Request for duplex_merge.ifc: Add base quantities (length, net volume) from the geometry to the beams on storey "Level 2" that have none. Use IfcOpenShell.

First a look at what the model holds.

```python
import ifcopenshell
import ifcopenshell.util.element
import ifcopenshell.util.unit

model = ifcopenshell.open("duplex_merge.ifc")
print(model.schema)
for unit_type in ("LENGTHUNIT", "AREAUNIT", "VOLUMEUNIT"):
    print(unit_type, ifcopenshell.util.unit.calculate_unit_scale(model, unit_type))
storey = next(s for s in model.by_type("IfcBuildingStorey") if s.Name == "Level 2")
beams = [e for e in ifcopenshell.util.element.get_decomposition(storey) if e.is_a("IfcBeam")]
for e in sorted(beams, key=lambda e: e.id()):
    print(e.id(), e.is_a(), e.Name, list(ifcopenshell.util.element.get_psets(e, qtos_only=True)), sep=" | ")
```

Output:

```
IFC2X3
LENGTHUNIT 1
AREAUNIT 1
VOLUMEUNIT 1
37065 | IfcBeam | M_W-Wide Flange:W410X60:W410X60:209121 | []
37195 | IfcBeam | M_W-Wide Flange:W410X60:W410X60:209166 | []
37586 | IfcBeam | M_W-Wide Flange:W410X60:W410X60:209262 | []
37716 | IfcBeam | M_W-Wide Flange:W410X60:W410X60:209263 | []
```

```python
import ifcopenshell
import ifcopenshell.api.pset
import ifcopenshell.geom
import ifcopenshell.util.element
import ifcopenshell.util.shape
import ifcopenshell.util.unit

model = ifcopenshell.open("duplex_merge.ifc")
unit_scale = ifcopenshell.util.unit.calculate_unit_scale(model)
volume_scale = ifcopenshell.util.unit.calculate_unit_scale(model, "VOLUMEUNIT")
settings = ifcopenshell.geom.settings()

storey = next(s for s in model.by_type("IfcBuildingStorey") if s.Name == "Level 2")
beams = [e for e in ifcopenshell.util.element.get_decomposition(storey) if e.is_a("IfcBeam")]

for e in sorted(beams, key=lambda e: e.id()):
    if ifcopenshell.util.element.get_psets(e, qtos_only=True, should_inherit=False):
        continue
    # Geometry comes back in metres, in the element's own axes.
    shape = ifcopenshell.geom.create_shape(settings, e)
    values = {
        "Length": ifcopenshell.util.shape.get_max_xyz(shape.geometry) / unit_scale,
        "NetVolume": ifcopenshell.util.shape.get_volume(shape.geometry) / volume_scale,
    }
    qto = ifcopenshell.api.pset.add_qto(model, product=e, name="BaseQuantities")
    ifcopenshell.api.pset.edit_qto(model, qto=qto, properties=values)
    print(e.id(), {k: round(v, 3) for k, v in values.items()})

model.write("duplex_merge_edited.ifc")
```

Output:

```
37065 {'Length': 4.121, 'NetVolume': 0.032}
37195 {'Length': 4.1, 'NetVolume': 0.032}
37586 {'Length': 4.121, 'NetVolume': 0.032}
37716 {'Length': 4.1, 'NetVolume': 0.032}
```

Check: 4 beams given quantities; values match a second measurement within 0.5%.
